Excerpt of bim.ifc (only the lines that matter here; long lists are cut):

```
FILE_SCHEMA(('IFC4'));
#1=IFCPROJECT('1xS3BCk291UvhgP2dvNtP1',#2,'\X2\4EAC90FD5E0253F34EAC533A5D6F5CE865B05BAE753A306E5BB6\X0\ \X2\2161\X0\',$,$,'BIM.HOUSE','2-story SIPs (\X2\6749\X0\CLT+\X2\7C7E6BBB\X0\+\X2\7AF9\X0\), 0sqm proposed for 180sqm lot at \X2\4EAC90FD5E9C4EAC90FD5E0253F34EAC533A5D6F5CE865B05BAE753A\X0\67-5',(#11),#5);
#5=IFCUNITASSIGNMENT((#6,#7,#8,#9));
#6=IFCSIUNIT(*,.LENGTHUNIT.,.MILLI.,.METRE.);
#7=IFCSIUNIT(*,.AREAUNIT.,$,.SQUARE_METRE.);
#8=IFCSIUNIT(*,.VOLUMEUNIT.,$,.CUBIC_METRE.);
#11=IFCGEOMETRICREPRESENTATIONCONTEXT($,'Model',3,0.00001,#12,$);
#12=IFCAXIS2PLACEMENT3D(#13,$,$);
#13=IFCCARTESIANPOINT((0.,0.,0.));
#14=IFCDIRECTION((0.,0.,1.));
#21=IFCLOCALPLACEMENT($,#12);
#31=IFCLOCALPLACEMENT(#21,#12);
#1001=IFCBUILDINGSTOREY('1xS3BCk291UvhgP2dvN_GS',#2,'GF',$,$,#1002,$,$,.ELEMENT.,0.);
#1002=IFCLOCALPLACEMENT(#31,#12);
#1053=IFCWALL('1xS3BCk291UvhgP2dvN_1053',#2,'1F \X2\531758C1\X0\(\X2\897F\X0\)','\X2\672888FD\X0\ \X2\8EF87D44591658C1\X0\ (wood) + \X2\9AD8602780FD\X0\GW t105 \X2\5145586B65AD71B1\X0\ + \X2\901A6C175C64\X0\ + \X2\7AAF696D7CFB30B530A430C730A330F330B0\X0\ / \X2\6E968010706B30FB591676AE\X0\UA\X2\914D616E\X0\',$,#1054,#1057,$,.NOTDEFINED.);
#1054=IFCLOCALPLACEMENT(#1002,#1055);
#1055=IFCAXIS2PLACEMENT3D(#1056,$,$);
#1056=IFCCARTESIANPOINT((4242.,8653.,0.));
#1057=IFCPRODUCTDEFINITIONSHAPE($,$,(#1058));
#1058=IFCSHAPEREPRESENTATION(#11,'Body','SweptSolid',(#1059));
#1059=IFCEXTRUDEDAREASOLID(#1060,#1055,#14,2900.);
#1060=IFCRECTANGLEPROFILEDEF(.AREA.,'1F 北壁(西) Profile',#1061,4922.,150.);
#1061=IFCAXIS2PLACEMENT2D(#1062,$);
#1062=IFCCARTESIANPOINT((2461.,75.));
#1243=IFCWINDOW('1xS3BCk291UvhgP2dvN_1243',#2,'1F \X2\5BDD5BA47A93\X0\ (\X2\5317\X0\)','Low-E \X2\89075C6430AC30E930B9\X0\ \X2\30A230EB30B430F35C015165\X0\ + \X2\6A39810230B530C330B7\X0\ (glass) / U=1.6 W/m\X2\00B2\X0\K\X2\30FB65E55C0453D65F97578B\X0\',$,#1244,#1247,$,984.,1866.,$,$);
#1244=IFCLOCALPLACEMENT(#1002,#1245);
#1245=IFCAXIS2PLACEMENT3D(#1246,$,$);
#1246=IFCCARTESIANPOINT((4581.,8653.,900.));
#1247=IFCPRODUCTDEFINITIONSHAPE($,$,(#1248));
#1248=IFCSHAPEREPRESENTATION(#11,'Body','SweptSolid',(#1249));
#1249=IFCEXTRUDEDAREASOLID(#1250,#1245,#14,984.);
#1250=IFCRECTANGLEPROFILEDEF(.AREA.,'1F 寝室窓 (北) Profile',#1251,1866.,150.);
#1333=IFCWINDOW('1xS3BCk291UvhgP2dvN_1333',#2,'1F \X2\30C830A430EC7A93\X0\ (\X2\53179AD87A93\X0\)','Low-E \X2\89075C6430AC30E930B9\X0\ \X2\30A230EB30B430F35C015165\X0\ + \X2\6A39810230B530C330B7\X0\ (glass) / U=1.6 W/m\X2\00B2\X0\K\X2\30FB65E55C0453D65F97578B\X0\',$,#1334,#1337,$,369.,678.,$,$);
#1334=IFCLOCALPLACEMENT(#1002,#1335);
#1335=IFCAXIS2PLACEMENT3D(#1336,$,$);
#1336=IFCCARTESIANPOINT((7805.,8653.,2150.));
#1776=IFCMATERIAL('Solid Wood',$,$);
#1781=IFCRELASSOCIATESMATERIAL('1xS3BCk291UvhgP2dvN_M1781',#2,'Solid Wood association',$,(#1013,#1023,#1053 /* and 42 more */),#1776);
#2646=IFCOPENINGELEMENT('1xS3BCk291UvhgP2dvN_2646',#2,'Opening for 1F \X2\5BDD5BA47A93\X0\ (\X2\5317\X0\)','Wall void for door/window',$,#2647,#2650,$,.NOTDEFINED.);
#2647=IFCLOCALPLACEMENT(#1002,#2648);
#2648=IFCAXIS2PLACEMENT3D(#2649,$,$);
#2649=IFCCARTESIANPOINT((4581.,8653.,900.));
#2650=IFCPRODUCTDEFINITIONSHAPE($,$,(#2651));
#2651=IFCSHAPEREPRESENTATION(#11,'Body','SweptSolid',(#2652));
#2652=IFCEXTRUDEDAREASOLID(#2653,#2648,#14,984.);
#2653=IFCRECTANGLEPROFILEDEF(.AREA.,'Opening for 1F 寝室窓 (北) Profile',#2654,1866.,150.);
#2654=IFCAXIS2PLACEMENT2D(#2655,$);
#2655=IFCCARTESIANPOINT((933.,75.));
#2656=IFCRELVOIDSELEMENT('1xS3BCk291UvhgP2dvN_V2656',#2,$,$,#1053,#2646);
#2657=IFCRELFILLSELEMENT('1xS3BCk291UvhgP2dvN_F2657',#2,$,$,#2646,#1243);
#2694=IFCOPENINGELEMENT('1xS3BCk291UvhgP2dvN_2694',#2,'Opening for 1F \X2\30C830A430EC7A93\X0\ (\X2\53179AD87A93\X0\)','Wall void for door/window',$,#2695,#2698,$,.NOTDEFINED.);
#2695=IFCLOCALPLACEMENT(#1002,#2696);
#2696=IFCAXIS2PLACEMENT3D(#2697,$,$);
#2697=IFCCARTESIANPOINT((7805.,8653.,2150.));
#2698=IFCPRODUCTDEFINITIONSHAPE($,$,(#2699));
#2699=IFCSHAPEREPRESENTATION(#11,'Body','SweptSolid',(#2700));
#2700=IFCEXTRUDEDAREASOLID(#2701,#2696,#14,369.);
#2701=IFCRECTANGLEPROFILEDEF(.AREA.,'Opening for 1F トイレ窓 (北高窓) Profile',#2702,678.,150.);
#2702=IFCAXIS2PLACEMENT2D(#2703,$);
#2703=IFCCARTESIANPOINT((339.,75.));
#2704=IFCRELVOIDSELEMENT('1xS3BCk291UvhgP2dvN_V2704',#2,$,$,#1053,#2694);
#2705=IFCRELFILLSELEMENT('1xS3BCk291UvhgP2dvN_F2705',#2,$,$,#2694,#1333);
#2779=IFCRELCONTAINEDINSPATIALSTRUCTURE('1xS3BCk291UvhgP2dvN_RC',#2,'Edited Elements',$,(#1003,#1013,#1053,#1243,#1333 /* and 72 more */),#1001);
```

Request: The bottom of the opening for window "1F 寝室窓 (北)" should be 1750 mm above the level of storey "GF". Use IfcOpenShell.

```python
import numpy as np
import ifcopenshell
import ifcopenshell.api.geometry
import ifcopenshell.geom
import ifcopenshell.util.element
import ifcopenshell.util.placement
import ifcopenshell.util.shape
import ifcopenshell.util.unit

model = ifcopenshell.open("bim.ifc")
unit_scale = ifcopenshell.util.unit.calculate_unit_scale(model)

window = model.by_guid("1xS3BCk291UvhgP2dvN_1243")
opening = window.FillsVoids[0].RelatingOpeningElement
storey = ifcopenshell.util.element.get_container(window, ifc_class="IfcBuildingStorey")
level = ifcopenshell.util.placement.get_local_placement(storey.ObjectPlacement)[2, 3]

# The opening's origin need not be at the sill, so measure its lowest point.
shape = ifcopenshell.geom.create_shape(ifcopenshell.geom.settings(), opening)
bottom = ifcopenshell.util.shape.get_shape_bottom_elevation(shape, shape.geometry) / unit_scale
dz = level + 1.75 / unit_scale - bottom

shift = np.array([0.0, 0.0, dz])
# The window is not placed relative to its opening, so move both.
for product in (opening, window):
    matrix = ifcopenshell.util.placement.get_local_placement(product.ObjectPlacement)
    matrix[:3, 3] += shift
    ifcopenshell.api.geometry.edit_object_placement(model, product=product, matrix=matrix, is_si=False)

print(f"moved by {dz * unit_scale:+.3f} m")

model.write("bim_updated.ifc")
```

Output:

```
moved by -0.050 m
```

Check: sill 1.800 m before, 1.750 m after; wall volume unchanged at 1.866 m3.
